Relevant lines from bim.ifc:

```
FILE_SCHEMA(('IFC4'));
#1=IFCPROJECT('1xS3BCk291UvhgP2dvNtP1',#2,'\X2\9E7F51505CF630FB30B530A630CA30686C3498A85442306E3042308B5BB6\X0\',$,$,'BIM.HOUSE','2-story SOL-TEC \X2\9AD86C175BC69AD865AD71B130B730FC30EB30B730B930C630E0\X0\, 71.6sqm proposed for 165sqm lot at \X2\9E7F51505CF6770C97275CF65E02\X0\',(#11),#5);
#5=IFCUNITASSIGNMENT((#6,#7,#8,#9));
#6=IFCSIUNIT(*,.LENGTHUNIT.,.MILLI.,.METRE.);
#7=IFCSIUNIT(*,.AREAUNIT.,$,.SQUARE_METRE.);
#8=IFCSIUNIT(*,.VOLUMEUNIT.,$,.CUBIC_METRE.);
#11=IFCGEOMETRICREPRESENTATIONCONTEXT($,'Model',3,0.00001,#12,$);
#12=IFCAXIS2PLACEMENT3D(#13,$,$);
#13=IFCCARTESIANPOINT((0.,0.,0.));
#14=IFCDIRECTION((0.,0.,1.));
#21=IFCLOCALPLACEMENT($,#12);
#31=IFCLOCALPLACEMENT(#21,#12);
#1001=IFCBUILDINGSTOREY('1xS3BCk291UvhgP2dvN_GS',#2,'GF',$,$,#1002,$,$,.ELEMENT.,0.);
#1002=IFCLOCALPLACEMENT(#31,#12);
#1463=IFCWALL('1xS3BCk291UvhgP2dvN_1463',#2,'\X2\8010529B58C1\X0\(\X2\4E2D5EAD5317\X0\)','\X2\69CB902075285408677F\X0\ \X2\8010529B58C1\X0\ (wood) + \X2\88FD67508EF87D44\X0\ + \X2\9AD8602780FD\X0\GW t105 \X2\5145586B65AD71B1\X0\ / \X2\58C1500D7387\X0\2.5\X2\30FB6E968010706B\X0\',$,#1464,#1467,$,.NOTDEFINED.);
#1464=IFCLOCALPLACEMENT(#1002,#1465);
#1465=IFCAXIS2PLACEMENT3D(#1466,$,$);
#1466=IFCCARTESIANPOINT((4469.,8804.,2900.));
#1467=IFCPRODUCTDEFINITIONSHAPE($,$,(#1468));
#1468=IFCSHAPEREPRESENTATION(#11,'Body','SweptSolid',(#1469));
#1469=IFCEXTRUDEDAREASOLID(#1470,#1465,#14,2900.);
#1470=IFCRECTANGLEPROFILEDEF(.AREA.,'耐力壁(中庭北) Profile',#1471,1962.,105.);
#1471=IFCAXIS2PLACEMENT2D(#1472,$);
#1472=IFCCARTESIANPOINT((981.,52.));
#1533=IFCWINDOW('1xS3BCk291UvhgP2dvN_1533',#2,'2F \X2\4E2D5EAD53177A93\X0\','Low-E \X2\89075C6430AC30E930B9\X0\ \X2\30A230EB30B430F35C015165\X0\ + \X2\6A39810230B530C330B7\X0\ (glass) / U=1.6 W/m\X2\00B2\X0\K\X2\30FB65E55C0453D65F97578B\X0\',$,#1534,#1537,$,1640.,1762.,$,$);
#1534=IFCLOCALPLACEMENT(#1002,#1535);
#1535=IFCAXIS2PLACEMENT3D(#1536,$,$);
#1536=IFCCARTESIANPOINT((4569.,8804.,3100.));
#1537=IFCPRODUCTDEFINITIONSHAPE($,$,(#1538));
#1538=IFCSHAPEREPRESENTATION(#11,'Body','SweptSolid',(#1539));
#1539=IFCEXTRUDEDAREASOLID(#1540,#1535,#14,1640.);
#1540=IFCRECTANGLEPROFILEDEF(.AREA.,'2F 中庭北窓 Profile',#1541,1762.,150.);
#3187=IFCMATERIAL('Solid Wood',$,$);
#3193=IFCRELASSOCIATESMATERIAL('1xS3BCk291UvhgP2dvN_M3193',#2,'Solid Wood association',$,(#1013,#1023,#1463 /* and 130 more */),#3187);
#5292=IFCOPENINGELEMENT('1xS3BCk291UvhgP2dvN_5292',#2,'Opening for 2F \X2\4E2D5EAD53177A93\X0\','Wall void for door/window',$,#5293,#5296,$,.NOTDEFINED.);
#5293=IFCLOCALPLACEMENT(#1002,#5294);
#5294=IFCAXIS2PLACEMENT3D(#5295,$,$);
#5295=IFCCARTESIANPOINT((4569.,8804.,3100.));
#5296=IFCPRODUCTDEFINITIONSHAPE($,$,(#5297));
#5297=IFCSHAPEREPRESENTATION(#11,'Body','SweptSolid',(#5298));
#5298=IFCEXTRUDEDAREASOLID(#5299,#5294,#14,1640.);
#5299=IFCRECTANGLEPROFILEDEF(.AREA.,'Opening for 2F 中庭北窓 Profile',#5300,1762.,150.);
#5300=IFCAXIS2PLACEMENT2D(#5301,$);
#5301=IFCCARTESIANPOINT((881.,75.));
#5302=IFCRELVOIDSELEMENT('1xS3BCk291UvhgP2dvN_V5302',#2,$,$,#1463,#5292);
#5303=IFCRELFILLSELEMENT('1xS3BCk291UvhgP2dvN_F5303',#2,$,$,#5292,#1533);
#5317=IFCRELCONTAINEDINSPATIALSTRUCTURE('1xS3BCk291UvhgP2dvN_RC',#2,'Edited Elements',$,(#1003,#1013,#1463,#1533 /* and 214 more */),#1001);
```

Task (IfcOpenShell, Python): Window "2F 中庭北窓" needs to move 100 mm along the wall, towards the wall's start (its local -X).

```python
import ifcopenshell
import ifcopenshell.api.geometry
import ifcopenshell.util.placement
import ifcopenshell.util.unit

model = ifcopenshell.open("bim.ifc")
unit_scale = ifcopenshell.util.unit.calculate_unit_scale(model)

window = model.by_id(1533)
opening = window.FillsVoids[0].RelatingOpeningElement
wall = opening.VoidsElements[0].RelatingBuildingElement

wall_matrix = ifcopenshell.util.placement.get_local_placement(wall.ObjectPlacement)
shift = wall_matrix[:3, 0] * -0.1 / unit_scale
before = ifcopenshell.util.placement.get_local_placement(window.ObjectPlacement)[:3, 3].copy()

# The window is not placed relative to its opening, so move both.
for product in (opening, window):
    matrix = ifcopenshell.util.placement.get_local_placement(product.ObjectPlacement)
    matrix[:3, 3] += shift
    ifcopenshell.api.geometry.edit_object_placement(model, product=product, matrix=matrix, is_si=False)

after = ifcopenshell.util.placement.get_local_placement(window.ObjectPlacement)[:3, 3]
print("window moved by", (after - before).round(3) + 0.0)

model.write("bim-out.ifc")
```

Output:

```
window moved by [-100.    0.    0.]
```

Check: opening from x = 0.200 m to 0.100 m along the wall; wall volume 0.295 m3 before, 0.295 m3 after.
